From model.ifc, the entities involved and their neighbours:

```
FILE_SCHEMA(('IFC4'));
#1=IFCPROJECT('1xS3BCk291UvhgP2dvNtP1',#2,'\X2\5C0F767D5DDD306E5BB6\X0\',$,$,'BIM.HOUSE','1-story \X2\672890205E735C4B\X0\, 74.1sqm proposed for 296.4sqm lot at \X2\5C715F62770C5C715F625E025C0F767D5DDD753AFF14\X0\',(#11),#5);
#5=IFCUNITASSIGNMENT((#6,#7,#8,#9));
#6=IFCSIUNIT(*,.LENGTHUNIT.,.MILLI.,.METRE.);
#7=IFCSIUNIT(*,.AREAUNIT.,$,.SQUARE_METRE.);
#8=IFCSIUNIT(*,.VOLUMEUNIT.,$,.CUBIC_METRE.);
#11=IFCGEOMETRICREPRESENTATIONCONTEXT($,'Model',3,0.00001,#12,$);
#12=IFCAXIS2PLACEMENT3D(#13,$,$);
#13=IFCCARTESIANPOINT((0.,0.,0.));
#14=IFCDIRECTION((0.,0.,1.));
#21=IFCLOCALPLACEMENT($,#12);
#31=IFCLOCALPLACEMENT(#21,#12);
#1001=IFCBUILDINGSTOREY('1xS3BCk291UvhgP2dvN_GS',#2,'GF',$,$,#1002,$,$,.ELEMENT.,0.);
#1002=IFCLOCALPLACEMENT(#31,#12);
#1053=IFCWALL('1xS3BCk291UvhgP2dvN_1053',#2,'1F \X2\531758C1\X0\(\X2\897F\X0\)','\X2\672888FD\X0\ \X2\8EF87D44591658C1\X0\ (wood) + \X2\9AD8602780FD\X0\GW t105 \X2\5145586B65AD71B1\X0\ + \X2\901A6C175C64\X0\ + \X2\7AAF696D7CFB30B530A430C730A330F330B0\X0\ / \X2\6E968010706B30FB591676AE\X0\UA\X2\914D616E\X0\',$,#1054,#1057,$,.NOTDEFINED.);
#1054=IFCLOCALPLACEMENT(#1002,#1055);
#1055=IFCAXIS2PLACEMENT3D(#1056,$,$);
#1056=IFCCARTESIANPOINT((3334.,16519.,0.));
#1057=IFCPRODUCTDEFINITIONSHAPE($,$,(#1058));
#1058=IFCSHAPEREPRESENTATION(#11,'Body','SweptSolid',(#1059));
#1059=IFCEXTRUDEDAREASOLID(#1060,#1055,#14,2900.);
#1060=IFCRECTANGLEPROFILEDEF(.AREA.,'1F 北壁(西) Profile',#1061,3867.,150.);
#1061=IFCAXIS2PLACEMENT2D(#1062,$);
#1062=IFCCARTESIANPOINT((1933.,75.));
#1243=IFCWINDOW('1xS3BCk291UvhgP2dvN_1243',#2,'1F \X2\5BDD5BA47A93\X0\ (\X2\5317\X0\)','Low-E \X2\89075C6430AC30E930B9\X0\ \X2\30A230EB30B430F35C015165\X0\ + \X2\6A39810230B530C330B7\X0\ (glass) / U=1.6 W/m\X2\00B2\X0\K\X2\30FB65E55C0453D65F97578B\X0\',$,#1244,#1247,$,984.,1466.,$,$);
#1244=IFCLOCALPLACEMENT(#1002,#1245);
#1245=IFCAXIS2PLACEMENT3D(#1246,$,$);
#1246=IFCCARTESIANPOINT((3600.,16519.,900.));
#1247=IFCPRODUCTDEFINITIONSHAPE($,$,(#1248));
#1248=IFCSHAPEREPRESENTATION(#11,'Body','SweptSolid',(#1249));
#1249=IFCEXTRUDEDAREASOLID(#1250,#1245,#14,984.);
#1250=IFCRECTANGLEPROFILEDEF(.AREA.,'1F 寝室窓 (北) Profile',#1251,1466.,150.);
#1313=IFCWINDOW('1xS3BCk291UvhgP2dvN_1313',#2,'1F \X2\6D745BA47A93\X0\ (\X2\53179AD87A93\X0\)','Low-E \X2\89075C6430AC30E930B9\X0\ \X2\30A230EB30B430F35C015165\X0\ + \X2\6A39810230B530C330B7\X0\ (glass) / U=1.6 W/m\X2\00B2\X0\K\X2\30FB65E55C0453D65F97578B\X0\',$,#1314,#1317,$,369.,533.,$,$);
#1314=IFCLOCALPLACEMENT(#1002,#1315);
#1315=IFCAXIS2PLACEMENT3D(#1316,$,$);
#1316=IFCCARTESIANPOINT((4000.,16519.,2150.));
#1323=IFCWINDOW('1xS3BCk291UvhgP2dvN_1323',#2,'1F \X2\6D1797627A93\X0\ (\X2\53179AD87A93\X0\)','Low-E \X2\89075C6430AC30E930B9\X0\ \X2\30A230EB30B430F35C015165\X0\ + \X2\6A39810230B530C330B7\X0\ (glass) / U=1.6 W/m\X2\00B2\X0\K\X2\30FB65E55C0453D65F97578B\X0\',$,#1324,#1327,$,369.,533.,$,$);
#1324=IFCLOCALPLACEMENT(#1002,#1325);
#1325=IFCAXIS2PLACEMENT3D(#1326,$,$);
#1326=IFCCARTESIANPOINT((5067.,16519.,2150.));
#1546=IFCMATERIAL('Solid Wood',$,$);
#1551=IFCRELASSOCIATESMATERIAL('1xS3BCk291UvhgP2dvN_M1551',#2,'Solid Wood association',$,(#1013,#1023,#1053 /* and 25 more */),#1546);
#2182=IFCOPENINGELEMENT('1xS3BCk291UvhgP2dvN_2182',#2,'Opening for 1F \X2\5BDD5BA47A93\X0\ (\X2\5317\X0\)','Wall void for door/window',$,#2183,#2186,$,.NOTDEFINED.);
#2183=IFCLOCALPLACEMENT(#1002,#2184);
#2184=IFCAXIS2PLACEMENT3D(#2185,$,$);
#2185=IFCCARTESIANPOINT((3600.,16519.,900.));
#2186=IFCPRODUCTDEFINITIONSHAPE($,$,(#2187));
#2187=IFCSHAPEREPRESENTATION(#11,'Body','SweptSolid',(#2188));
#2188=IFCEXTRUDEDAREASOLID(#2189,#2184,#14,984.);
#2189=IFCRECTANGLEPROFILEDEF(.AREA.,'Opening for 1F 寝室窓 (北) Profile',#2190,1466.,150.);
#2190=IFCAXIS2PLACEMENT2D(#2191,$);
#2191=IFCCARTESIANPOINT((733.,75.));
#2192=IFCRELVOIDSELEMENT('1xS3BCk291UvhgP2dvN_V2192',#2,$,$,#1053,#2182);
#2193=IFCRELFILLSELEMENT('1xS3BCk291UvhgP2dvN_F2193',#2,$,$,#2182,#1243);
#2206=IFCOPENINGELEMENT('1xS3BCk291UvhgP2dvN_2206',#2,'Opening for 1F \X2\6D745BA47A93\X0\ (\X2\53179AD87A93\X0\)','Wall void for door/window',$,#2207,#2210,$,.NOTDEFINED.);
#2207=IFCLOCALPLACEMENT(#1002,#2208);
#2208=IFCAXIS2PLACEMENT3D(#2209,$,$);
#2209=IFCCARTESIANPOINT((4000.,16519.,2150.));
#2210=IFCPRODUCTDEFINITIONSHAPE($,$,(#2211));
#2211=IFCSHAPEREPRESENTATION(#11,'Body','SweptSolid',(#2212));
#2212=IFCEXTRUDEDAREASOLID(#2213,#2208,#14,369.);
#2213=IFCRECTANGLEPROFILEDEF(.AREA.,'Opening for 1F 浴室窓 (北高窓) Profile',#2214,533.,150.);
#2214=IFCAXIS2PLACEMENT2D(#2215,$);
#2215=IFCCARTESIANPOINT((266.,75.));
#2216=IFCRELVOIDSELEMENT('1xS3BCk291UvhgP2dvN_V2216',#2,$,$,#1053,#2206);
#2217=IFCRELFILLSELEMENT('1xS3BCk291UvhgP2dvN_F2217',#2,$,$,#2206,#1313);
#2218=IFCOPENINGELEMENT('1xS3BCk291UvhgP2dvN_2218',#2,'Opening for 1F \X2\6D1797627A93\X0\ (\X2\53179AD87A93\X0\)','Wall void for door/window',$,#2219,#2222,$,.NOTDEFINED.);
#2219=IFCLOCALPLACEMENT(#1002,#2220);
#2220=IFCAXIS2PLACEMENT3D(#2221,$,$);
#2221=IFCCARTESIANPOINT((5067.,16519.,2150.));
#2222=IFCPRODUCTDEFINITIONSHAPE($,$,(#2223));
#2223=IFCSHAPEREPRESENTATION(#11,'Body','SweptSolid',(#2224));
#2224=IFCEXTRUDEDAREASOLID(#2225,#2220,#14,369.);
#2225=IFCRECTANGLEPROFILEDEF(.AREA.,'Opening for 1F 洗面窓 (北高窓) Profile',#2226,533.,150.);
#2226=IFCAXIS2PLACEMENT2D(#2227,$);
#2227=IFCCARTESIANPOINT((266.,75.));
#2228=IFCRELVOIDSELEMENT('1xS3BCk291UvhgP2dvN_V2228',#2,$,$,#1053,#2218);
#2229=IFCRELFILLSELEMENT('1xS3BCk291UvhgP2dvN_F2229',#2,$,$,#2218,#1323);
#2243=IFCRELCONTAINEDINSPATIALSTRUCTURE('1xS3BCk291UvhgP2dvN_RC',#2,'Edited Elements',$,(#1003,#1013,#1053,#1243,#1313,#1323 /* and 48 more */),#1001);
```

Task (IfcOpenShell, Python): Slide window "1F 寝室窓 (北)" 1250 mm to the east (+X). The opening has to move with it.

```python
import ifcopenshell
import ifcopenshell.api.geometry
import ifcopenshell.util.placement
import ifcopenshell.util.unit

model = ifcopenshell.open("model.ifc")
unit_scale = ifcopenshell.util.unit.calculate_unit_scale(model)

window = model.by_guid("1xS3BCk291UvhgP2dvN_1243")
opening = window.FillsVoids[0].RelatingOpeningElement
wall = opening.VoidsElements[0].RelatingBuildingElement

wall_matrix = ifcopenshell.util.placement.get_local_placement(wall.ObjectPlacement)
shift = wall_matrix[:3, 0] * 1.25 / unit_scale
before = ifcopenshell.util.placement.get_local_placement(window.ObjectPlacement)[:3, 3].copy()

# The window is not placed relative to its opening, so move both.
for product in (opening, window):
    matrix = ifcopenshell.util.placement.get_local_placement(product.ObjectPlacement)
    matrix[:3, 3] += shift
    ifcopenshell.api.geometry.edit_object_placement(model, product=product, matrix=matrix, is_si=False)

after = ifcopenshell.util.placement.get_local_placement(window.ObjectPlacement)[:3, 3]
print("window moved by", (after - before).round(3) + 0.0)

model.write("model_edited.ifc")
```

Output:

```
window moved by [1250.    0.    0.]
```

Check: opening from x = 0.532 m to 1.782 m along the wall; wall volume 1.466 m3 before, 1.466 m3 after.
